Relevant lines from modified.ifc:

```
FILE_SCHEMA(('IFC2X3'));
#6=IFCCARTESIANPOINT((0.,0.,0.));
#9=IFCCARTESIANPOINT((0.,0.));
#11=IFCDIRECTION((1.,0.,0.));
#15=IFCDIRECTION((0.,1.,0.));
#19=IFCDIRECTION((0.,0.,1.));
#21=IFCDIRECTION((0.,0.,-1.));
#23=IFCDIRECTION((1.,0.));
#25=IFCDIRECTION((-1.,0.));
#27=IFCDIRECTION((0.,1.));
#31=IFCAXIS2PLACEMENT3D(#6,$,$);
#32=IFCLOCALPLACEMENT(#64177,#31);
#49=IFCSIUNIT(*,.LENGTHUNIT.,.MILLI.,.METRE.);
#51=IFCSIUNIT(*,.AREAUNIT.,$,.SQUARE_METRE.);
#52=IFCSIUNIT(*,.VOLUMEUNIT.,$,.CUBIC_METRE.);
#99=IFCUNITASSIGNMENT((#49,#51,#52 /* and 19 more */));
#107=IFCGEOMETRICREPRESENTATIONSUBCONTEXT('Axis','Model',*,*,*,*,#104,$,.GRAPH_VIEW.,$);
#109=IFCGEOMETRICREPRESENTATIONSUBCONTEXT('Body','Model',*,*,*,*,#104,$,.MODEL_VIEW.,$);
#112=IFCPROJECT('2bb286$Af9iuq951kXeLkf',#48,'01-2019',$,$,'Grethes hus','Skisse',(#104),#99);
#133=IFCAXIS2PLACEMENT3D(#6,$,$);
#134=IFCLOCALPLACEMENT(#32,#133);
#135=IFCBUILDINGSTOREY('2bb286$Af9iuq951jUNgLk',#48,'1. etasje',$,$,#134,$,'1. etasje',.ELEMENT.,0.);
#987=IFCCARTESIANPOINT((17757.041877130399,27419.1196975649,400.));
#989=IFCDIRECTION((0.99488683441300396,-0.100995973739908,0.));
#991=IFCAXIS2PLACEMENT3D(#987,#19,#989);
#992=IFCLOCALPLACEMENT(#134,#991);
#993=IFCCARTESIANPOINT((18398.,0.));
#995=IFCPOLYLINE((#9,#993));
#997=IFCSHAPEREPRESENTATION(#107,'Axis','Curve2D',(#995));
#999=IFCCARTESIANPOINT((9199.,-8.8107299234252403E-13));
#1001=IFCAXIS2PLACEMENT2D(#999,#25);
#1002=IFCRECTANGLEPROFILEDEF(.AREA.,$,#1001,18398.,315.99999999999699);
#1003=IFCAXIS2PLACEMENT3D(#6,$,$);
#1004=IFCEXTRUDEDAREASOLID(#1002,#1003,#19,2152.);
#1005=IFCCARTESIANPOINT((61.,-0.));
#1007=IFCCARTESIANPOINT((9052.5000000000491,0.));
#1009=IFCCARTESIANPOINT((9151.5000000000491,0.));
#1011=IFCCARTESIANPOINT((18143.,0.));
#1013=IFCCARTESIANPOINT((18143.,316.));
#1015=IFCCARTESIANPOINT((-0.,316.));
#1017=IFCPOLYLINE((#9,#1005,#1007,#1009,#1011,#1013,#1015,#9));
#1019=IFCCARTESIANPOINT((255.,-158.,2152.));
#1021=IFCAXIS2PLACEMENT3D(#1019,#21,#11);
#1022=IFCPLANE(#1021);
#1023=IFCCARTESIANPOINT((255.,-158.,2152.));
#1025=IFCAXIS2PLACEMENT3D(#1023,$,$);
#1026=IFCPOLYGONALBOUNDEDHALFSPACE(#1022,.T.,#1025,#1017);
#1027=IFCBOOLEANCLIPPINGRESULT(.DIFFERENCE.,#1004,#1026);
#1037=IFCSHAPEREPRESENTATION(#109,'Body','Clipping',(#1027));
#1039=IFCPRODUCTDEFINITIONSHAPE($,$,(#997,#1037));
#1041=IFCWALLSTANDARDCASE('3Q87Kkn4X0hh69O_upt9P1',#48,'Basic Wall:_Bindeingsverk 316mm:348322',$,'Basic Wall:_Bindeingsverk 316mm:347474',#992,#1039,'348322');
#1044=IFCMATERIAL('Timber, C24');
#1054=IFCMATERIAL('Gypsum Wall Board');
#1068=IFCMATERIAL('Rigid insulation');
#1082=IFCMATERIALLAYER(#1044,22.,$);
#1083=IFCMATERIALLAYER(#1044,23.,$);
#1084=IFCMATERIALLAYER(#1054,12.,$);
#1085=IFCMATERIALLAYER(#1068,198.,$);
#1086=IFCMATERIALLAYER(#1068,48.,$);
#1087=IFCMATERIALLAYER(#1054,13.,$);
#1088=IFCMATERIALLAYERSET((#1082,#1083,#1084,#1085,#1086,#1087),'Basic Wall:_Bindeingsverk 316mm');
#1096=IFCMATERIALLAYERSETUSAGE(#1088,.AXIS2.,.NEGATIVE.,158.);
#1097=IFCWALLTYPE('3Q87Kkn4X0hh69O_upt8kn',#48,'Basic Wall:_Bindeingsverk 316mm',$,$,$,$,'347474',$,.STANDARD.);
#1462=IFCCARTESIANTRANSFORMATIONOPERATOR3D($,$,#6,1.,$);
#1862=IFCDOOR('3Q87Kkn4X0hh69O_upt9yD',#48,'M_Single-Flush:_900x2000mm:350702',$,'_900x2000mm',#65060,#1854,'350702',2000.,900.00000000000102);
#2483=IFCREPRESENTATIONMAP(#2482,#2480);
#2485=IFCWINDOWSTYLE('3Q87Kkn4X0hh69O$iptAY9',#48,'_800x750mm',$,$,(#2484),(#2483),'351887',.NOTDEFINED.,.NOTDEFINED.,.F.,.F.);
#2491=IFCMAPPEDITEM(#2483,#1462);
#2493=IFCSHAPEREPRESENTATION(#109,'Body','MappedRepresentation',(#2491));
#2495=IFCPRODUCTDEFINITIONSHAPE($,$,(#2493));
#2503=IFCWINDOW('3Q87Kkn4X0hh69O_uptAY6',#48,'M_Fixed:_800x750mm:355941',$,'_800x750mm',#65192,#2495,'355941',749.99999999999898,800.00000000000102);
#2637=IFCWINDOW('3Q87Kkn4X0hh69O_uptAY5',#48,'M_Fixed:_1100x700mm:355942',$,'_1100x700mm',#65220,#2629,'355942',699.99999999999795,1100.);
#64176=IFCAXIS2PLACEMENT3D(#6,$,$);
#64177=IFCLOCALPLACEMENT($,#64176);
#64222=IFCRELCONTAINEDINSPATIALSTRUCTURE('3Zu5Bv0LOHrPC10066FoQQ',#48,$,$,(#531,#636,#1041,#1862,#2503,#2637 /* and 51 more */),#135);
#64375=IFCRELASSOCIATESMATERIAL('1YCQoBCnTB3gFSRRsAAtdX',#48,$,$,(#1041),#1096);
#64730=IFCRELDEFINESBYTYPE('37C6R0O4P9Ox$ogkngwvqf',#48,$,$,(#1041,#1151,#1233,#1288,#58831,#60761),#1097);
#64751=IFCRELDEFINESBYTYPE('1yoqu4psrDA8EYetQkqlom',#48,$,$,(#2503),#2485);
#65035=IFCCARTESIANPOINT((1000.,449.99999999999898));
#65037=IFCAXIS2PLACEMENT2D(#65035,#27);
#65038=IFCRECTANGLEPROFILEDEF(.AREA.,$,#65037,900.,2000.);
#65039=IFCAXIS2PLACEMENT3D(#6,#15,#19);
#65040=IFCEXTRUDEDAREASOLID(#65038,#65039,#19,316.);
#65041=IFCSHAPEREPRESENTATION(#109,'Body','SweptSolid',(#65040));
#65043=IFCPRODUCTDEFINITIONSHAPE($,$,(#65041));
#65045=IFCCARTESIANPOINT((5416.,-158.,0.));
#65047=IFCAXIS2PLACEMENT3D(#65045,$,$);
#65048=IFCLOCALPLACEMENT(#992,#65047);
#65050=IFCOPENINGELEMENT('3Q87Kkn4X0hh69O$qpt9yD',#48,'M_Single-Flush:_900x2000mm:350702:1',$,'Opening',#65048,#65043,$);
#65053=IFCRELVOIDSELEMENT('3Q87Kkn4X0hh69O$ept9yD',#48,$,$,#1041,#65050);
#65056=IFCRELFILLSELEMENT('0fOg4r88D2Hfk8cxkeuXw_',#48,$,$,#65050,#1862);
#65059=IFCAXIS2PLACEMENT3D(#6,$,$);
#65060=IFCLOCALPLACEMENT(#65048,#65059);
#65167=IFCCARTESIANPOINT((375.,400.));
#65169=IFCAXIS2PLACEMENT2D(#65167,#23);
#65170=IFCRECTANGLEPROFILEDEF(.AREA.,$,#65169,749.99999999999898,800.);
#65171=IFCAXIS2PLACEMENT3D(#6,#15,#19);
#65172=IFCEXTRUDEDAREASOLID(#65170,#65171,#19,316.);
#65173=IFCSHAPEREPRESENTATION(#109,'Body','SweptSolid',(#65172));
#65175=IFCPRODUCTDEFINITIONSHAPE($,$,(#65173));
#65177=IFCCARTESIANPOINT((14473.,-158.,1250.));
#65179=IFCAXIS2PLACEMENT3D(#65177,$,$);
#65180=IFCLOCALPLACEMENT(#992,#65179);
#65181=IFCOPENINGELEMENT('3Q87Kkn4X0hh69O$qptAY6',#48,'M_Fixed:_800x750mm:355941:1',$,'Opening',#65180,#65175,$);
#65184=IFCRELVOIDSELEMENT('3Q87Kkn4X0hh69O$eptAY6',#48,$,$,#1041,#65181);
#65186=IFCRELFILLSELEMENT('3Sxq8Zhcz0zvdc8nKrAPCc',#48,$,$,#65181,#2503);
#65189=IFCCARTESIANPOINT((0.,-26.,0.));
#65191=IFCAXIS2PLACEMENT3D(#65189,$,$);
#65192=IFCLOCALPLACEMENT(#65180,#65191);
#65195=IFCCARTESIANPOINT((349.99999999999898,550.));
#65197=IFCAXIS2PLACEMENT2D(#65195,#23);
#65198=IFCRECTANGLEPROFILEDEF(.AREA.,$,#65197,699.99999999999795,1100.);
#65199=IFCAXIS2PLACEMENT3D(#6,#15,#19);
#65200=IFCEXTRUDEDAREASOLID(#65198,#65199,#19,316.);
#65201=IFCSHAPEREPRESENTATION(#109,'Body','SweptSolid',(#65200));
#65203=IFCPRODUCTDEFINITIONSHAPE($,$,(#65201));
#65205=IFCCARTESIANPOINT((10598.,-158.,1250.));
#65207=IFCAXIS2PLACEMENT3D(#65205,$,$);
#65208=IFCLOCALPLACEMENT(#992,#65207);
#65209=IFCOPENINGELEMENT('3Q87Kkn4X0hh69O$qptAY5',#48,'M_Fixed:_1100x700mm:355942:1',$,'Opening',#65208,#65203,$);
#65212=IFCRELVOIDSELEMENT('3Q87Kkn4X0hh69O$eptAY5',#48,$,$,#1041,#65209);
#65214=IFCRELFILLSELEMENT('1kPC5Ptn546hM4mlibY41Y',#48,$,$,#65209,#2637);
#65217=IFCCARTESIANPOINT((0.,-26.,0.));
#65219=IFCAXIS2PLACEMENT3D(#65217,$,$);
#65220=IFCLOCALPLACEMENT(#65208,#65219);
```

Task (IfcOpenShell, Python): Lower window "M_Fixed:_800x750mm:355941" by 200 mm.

```python
import numpy as np
import ifcopenshell
import ifcopenshell.api.geometry
import ifcopenshell.util.placement
import ifcopenshell.util.unit

model = ifcopenshell.open("modified.ifc")
unit_scale = ifcopenshell.util.unit.calculate_unit_scale(model)

window = model.by_guid("3Q87Kkn4X0hh69O_uptAY6")
opening = window.FillsVoids[0].RelatingOpeningElement
dz = -0.2 / unit_scale

shift = np.array([0.0, 0.0, dz])
# The window is placed relative to its opening, so it follows when the opening moves.
matrix = ifcopenshell.util.placement.get_local_placement(opening.ObjectPlacement)
matrix[:3, 3] += shift
ifcopenshell.api.geometry.edit_object_placement(
    model, product=opening, matrix=matrix, is_si=False, should_transform_children=True
)

print(f"moved by {dz * unit_scale:+.3f} m")

model.write("modified_rev.ifc")
```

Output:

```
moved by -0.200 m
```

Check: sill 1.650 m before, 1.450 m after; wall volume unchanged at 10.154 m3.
